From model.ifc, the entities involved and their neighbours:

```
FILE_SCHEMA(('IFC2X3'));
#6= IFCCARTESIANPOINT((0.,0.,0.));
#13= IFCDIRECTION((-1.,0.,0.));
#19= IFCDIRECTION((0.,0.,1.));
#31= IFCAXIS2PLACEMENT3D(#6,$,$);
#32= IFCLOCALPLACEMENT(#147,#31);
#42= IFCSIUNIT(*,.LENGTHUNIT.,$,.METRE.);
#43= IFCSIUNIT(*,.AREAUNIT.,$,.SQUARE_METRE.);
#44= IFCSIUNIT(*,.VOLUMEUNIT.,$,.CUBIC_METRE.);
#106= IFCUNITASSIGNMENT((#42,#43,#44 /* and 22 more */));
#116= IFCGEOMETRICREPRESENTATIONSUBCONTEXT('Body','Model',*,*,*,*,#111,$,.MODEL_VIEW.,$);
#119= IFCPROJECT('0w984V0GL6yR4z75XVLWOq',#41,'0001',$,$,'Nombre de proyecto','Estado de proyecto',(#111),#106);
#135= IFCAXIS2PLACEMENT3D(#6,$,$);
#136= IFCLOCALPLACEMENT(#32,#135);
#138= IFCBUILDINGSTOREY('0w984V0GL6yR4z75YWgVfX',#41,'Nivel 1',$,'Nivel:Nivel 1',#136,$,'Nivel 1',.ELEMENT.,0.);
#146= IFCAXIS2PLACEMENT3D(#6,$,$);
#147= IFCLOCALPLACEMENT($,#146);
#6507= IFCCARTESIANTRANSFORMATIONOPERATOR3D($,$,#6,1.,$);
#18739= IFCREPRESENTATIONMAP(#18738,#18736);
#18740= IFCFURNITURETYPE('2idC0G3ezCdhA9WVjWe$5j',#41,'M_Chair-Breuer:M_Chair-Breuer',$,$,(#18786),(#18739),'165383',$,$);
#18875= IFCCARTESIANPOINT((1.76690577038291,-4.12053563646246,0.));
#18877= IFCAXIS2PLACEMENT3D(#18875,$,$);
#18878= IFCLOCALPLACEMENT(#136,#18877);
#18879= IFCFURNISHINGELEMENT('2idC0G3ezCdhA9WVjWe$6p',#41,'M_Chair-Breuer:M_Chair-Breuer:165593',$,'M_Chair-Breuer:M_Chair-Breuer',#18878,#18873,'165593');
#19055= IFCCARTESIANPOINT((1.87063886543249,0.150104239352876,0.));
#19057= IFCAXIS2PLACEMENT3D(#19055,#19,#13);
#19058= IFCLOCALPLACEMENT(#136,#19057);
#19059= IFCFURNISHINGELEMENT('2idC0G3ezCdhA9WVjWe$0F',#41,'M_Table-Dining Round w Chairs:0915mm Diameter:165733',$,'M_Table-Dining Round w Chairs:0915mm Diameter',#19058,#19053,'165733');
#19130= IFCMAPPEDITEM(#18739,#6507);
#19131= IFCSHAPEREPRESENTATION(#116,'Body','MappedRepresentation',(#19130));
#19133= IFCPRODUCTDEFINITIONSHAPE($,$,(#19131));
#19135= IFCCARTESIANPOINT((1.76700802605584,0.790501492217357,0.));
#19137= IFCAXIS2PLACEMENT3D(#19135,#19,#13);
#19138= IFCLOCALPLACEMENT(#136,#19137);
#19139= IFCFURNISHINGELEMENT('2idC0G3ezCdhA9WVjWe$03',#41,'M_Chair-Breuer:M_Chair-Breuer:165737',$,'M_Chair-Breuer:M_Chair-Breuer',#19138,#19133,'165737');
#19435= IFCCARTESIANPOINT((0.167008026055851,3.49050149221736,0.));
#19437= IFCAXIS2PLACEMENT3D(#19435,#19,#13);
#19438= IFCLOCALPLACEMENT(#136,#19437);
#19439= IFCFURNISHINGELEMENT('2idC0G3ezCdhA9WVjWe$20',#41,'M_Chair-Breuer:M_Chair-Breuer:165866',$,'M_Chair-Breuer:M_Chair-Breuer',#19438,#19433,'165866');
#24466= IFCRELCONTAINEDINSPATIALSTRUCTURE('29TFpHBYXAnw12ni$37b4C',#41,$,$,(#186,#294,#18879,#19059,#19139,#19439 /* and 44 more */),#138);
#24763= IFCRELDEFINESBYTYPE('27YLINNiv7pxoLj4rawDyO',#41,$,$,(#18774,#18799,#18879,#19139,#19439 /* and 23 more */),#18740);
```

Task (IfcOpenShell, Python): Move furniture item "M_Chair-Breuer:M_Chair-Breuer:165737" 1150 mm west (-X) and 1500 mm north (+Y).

```python
import ifcopenshell
import ifcopenshell.api.geometry
import ifcopenshell.util.placement
import ifcopenshell.util.unit

model = ifcopenshell.open("model.ifc")
unit_scale = ifcopenshell.util.unit.calculate_unit_scale(model)

item = model.by_guid("2idC0G3ezCdhA9WVjWe$03")
matrix = ifcopenshell.util.placement.get_local_placement(item.ObjectPlacement)
matrix[0, 3] -= 1.15 / unit_scale
matrix[1, 3] += 1.5 / unit_scale
ifcopenshell.api.geometry.edit_object_placement(model, product=item, matrix=matrix, is_si=False)

print(ifcopenshell.util.placement.get_local_placement(item.ObjectPlacement).round(3) + 0.0)

model.write("model_v2.ifc")
```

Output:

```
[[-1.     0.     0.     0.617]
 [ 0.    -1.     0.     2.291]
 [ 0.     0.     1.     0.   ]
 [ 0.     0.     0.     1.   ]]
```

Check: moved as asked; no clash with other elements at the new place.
